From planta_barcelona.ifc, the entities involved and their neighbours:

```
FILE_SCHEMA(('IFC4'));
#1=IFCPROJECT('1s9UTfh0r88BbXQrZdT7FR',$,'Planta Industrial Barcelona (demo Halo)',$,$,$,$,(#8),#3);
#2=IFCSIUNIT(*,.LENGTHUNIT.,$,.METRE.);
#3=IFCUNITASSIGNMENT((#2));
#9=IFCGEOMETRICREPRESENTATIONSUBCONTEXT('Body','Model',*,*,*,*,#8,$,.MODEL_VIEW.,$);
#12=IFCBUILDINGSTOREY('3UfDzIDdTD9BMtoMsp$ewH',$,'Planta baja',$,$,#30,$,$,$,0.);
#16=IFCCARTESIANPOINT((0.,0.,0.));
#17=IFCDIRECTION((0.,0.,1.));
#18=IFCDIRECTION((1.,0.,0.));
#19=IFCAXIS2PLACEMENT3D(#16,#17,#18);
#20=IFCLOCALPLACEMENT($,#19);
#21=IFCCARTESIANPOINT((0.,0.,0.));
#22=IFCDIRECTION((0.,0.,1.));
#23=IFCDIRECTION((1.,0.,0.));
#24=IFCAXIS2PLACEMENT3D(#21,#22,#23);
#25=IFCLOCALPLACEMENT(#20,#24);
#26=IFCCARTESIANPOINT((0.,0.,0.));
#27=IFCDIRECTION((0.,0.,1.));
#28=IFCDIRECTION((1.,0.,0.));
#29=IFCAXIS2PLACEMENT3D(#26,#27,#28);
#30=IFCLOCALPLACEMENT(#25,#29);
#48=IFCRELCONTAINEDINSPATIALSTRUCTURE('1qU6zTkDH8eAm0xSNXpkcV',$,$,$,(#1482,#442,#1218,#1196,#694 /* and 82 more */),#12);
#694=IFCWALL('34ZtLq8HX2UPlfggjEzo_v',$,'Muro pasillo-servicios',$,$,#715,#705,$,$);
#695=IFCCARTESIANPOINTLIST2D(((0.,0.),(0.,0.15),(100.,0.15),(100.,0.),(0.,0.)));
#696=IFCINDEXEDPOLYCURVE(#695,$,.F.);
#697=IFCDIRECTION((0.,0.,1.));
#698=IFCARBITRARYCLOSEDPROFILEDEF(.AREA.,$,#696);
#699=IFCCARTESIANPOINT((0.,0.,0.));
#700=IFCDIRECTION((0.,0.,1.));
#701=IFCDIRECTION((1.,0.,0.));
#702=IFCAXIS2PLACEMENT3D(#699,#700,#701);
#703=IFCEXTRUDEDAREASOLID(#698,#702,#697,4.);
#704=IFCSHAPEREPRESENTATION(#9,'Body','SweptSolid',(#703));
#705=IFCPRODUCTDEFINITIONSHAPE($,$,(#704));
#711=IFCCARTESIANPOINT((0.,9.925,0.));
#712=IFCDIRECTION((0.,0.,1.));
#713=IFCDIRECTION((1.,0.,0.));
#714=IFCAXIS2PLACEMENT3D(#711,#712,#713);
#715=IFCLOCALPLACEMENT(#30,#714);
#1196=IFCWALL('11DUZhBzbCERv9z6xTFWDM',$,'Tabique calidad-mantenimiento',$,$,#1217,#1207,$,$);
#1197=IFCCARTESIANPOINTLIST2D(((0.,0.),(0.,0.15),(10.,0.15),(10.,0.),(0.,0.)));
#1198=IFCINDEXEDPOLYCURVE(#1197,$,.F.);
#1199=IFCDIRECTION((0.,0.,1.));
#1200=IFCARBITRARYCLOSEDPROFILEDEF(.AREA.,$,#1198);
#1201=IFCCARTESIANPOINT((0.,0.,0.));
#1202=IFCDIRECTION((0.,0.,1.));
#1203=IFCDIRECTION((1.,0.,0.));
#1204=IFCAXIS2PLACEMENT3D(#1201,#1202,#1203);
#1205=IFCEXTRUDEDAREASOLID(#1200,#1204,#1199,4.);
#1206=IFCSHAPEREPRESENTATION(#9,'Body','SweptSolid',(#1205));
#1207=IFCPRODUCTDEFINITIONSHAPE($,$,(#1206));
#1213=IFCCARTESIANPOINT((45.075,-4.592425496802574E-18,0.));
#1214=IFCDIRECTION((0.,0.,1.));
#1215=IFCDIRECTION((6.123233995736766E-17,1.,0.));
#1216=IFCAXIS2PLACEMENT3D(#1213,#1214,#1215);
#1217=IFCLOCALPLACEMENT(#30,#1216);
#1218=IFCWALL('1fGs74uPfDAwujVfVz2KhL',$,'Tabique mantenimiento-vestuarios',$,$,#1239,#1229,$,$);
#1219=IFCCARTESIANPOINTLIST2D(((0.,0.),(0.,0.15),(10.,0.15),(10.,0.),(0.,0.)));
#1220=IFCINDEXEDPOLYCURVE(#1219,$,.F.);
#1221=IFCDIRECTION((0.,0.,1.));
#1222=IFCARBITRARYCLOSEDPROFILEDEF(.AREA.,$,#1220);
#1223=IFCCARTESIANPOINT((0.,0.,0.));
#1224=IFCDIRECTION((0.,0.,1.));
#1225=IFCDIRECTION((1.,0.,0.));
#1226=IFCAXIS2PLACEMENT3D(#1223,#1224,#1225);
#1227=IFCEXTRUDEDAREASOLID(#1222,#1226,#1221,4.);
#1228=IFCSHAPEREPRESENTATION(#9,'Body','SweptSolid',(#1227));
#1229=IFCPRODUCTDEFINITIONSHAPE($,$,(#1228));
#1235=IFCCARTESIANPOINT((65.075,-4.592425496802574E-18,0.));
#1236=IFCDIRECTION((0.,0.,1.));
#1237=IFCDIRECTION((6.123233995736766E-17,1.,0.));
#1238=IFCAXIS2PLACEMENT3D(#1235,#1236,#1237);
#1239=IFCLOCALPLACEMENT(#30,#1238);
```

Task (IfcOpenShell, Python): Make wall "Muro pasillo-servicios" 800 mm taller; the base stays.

```python
import ifcopenshell
import ifcopenshell.geom
import ifcopenshell.util.representation
import ifcopenshell.util.shape
import ifcopenshell.util.unit

model = ifcopenshell.open("planta_barcelona.ifc")
unit_scale = ifcopenshell.util.unit.calculate_unit_scale(model)
settings = ifcopenshell.geom.settings()


def volume(element):
    """Net volume in cubic metres, openings subtracted."""
    shape = ifcopenshell.geom.create_shape(settings, element)
    return ifcopenshell.util.shape.get_volume(shape.geometry)


wall = model.by_id(694)
before = volume(wall)

body = ifcopenshell.util.representation.get_representation(wall, "Model", "Body")
solid = body.Items[0]
old_height = solid.Depth
solid.Depth += 0.8 / unit_scale
after = volume(wall)

print(f"height {old_height:g} -> {solid.Depth:g}, volume {before:.3f} -> {after:.3f} m3")

model.write("planta_barcelona-out.ifc")
```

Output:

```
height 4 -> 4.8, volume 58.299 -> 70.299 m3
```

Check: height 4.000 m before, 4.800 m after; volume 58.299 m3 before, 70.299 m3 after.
